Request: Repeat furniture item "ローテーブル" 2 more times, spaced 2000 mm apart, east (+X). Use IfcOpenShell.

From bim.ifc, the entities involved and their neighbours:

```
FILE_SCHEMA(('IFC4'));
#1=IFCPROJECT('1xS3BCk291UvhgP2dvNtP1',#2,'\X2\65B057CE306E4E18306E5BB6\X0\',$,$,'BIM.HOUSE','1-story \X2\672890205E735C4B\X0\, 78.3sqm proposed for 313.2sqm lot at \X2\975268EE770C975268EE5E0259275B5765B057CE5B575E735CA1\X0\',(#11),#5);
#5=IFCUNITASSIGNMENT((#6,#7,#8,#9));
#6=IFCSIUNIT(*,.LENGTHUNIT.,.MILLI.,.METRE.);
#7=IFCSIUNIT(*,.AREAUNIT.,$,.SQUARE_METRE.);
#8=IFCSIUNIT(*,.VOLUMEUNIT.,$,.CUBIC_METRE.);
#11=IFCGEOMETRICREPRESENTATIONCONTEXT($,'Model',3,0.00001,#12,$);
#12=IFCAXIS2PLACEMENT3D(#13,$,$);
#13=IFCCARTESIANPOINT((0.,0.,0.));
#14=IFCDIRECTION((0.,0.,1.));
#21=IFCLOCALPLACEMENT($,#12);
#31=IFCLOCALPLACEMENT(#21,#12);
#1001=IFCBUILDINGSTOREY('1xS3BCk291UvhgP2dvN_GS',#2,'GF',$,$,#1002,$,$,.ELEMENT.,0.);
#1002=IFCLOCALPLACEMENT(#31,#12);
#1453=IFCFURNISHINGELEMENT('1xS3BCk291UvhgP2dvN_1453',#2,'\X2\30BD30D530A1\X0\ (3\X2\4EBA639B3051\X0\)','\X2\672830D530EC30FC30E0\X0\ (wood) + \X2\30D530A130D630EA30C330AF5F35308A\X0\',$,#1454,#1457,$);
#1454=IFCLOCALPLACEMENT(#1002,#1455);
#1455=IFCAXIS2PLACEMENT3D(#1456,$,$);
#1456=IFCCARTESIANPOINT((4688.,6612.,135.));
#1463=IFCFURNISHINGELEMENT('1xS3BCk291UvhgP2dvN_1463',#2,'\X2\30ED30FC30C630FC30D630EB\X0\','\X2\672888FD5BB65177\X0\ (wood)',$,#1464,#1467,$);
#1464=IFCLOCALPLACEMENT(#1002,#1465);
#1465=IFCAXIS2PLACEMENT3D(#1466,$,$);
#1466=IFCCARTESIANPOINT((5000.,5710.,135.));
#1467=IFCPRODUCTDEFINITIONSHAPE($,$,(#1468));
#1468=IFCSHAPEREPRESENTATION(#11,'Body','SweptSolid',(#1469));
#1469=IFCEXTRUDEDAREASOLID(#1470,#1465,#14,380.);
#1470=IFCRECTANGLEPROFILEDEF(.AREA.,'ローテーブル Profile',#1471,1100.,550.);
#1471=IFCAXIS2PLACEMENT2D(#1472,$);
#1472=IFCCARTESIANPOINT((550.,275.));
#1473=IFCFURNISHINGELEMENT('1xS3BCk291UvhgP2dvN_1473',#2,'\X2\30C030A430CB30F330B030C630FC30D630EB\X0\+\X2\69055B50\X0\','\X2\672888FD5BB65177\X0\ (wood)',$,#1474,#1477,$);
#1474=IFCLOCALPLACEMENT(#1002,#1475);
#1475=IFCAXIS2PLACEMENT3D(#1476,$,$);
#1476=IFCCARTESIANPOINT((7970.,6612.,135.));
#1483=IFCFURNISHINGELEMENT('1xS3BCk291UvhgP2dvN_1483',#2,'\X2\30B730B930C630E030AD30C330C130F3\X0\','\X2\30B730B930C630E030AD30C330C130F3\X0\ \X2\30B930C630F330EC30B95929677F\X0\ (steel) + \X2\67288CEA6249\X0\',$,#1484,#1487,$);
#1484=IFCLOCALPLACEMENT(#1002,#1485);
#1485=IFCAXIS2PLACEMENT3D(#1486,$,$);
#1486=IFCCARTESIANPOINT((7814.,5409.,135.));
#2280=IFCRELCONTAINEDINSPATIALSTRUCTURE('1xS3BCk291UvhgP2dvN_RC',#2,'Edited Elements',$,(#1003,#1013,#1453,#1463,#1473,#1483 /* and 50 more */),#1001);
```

```python
import numpy as np
import ifcopenshell
import ifcopenshell.api.geometry
import ifcopenshell.api.root
import ifcopenshell.util.element
import ifcopenshell.util.placement
import ifcopenshell.util.unit

model = ifcopenshell.open("bim.ifc")
unit_scale = ifcopenshell.util.unit.calculate_unit_scale(model)


def reuse_history(source, copy):
    """copy_class also copies each property set's owner history, people and application; keep the originals."""
    for rel in copy.IsDefinedBy:
        if rel.is_a("IfcRelDefinesByProperties") and (history := rel.RelatingPropertyDefinition.OwnerHistory):
            rel.RelatingPropertyDefinition.OwnerHistory = source.OwnerHistory
            ifcopenshell.util.element.remove_deep2(model, history)


source = model.by_guid("1xS3BCk291UvhgP2dvN_1463")
base = ifcopenshell.util.placement.get_local_placement(source.ObjectPlacement)
step = np.array([1.0, 0.0, 0.0]) * 2 / unit_scale

for i in range(1, 3):
    copy = ifcopenshell.api.root.copy_class(model, product=source)
    copy.Representation = ifcopenshell.util.element.copy_deep(
        model, source.Representation, exclude=["IfcGeometricRepresentationContext", "IfcRepresentationMap"]
    )
    reuse_history(source, copy)
    matrix = base.copy()
    matrix[:3, 3] += i * step
    print("added at", matrix[:3, 3].round(3) + 0.0)
    ifcopenshell.api.geometry.edit_object_placement(model, product=copy, matrix=matrix, is_si=False)

model.write("bim_rev.ifc")
```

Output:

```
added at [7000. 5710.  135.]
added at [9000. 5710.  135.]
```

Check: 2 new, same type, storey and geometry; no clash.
